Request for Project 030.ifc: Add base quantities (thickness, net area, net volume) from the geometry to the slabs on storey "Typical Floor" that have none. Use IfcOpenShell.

First a look at what the model holds.

```python
import ifcopenshell
import ifcopenshell.util.element
import ifcopenshell.util.unit

model = ifcopenshell.open("Project 030.ifc")
print(model.schema)
for unit_type in ("LENGTHUNIT", "AREAUNIT", "VOLUMEUNIT"):
    print(unit_type, ifcopenshell.util.unit.calculate_unit_scale(model, unit_type))
storey = next(s for s in model.by_type("IfcBuildingStorey") if s.Name == "Typical Floor")
slabs = [e for e in ifcopenshell.util.element.get_decomposition(storey) if e.is_a("IfcSlab")]
for e in sorted(slabs, key=lambda e: e.id()):
    print(e.id(), e.is_a(), e.Name, list(ifcopenshell.util.element.get_psets(e, qtos_only=True)), sep=" | ")
```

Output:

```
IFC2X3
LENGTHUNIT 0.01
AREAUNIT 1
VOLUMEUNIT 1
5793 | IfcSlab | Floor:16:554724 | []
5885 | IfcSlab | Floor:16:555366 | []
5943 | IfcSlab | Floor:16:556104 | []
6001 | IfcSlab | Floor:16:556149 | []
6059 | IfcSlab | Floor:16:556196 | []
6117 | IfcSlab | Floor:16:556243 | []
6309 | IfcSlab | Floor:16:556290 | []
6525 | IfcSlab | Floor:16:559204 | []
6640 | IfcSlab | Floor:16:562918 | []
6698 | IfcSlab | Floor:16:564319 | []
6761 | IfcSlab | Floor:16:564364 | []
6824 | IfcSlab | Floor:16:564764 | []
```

```python
import ifcopenshell
import ifcopenshell.api.pset
import ifcopenshell.geom
import ifcopenshell.util.element
import ifcopenshell.util.shape
import ifcopenshell.util.unit

model = ifcopenshell.open("Project 030.ifc")
unit_scale = ifcopenshell.util.unit.calculate_unit_scale(model)
area_scale = ifcopenshell.util.unit.calculate_unit_scale(model, "AREAUNIT")
volume_scale = ifcopenshell.util.unit.calculate_unit_scale(model, "VOLUMEUNIT")
settings = ifcopenshell.geom.settings()

storey = next(s for s in model.by_type("IfcBuildingStorey") if s.Name == "Typical Floor")
slabs = [e for e in ifcopenshell.util.element.get_decomposition(storey) if e.is_a("IfcSlab")]

for e in sorted(slabs, key=lambda e: e.id()):
    if ifcopenshell.util.element.get_psets(e, qtos_only=True, should_inherit=False):
        continue
    # Geometry comes back in metres, in the element's own axes.
    shape = ifcopenshell.geom.create_shape(settings, e)
    values = {
        "Width": ifcopenshell.util.shape.get_z(shape.geometry) / unit_scale,
        "NetArea": ifcopenshell.util.shape.get_footprint_area(shape.geometry) / area_scale,
        "NetVolume": ifcopenshell.util.shape.get_volume(shape.geometry) / volume_scale,
    }
    qto = ifcopenshell.api.pset.add_qto(model, product=e, name="BaseQuantities")
    ifcopenshell.api.pset.edit_qto(model, qto=qto, properties=values)
    print(e.id(), {k: round(v, 3) for k, v in values.items()})

model.write("Project 030-out.ifc")
```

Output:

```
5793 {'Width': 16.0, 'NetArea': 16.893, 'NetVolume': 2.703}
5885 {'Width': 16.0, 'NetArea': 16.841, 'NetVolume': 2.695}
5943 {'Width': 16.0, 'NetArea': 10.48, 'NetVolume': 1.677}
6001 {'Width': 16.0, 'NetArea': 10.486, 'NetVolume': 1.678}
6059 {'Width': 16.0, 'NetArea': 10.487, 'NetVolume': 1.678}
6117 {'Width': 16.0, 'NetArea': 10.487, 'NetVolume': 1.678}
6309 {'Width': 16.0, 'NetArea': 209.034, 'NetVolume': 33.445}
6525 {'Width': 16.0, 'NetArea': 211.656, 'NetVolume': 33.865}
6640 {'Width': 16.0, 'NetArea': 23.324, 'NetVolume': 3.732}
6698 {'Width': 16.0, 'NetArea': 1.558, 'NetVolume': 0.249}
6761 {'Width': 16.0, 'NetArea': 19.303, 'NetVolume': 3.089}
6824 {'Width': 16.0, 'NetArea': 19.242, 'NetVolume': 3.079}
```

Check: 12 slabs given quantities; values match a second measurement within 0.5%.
